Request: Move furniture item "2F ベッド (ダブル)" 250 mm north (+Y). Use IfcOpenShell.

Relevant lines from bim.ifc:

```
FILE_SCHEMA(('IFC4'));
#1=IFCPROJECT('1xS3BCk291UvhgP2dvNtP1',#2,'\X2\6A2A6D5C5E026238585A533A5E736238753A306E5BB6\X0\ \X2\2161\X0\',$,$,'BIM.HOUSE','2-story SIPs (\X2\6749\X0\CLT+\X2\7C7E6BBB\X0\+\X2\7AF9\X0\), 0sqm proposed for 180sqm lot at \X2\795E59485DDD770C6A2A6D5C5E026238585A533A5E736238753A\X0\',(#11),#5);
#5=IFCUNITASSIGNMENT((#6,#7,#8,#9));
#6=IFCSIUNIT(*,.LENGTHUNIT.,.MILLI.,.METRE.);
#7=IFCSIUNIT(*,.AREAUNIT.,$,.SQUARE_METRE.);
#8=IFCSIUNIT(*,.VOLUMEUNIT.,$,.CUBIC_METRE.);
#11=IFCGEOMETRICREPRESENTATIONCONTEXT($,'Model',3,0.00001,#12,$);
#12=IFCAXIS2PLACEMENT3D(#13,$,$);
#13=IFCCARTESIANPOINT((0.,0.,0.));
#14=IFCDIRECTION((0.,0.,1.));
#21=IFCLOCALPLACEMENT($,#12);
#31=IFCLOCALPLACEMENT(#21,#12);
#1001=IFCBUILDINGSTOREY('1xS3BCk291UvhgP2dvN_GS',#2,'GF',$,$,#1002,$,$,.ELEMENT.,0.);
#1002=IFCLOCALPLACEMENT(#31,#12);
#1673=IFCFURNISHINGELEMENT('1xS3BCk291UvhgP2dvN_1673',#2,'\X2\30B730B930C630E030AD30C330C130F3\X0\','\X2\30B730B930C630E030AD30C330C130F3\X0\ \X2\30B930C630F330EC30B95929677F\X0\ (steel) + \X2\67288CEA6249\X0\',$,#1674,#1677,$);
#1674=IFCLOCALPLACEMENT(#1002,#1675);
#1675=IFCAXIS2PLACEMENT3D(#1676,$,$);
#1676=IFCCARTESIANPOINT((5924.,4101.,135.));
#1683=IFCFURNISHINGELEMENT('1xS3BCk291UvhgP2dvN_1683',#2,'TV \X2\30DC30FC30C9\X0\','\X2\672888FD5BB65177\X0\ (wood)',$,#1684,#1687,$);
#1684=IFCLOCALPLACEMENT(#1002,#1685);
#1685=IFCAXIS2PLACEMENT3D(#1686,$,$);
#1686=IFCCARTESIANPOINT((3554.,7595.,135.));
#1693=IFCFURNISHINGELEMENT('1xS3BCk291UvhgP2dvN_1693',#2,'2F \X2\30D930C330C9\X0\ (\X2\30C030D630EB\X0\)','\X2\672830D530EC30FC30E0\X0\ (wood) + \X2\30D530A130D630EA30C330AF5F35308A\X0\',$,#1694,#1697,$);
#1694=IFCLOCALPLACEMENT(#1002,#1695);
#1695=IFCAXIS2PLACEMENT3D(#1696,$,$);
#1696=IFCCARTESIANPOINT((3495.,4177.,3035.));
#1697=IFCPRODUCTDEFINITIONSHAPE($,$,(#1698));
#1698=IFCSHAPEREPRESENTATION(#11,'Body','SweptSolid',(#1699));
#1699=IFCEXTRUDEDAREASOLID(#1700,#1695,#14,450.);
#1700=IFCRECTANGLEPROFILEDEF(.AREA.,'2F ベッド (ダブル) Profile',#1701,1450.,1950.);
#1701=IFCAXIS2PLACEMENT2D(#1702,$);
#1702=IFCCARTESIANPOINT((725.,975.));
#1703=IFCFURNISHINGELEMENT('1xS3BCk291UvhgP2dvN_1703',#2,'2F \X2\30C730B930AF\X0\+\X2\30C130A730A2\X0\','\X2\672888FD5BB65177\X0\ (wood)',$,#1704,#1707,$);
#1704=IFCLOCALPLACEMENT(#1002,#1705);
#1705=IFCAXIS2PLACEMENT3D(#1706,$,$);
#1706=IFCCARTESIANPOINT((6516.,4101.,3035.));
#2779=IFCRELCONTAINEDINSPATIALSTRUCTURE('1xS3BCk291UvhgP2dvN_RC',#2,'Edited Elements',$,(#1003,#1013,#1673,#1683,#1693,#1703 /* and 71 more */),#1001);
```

```python
import ifcopenshell
import ifcopenshell.api.geometry
import ifcopenshell.util.placement

model = ifcopenshell.open("bim.ifc")

item = model.by_guid("1xS3BCk291UvhgP2dvN_1693")
matrix = ifcopenshell.util.placement.get_local_placement(item.ObjectPlacement)
matrix[1, 3] += 250.0
ifcopenshell.api.geometry.edit_object_placement(model, product=item, matrix=matrix, is_si=False)

print(ifcopenshell.util.placement.get_local_placement(item.ObjectPlacement).round(3) + 0.0)

model.write("bim_updated.ifc")
```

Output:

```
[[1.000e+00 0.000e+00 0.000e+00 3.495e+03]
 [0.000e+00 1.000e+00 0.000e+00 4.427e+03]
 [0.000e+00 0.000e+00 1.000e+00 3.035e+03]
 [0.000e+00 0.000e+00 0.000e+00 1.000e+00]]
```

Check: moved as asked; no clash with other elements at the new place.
